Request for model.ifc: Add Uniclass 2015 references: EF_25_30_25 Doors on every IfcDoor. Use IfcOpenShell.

First a look at what the model holds.

```python
import ifcopenshell

model = ifcopenshell.open("model.ifc")
print(model.schema)
print("classifications:", [c.Name for c in model.by_type("IfcClassification")])
for ifc_class in ("IfcDoor", "IfcRoof", "IfcStair", "IfcWall", "IfcWindow"):
    print(ifc_class, len(model.by_type(ifc_class)))
```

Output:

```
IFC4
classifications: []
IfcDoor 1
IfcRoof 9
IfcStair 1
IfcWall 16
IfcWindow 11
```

```python
import ifcopenshell
import ifcopenshell.api.classification

model = ifcopenshell.open("model.ifc")

system = ifcopenshell.api.classification.add_classification(model, classification="Uniclass 2015")

codes = {
    "IfcDoor": ("EF_25_30_25", "Doors"),
}
for ifc_class, (code, name) in codes.items():
    products = model.by_type(ifc_class)
    ifcopenshell.api.classification.add_reference(
        model, products=products, classification=system, identification=code, name=name
    )
    print(code, len(products))

model.write("model_updated.ifc")
```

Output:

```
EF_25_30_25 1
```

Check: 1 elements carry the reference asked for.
